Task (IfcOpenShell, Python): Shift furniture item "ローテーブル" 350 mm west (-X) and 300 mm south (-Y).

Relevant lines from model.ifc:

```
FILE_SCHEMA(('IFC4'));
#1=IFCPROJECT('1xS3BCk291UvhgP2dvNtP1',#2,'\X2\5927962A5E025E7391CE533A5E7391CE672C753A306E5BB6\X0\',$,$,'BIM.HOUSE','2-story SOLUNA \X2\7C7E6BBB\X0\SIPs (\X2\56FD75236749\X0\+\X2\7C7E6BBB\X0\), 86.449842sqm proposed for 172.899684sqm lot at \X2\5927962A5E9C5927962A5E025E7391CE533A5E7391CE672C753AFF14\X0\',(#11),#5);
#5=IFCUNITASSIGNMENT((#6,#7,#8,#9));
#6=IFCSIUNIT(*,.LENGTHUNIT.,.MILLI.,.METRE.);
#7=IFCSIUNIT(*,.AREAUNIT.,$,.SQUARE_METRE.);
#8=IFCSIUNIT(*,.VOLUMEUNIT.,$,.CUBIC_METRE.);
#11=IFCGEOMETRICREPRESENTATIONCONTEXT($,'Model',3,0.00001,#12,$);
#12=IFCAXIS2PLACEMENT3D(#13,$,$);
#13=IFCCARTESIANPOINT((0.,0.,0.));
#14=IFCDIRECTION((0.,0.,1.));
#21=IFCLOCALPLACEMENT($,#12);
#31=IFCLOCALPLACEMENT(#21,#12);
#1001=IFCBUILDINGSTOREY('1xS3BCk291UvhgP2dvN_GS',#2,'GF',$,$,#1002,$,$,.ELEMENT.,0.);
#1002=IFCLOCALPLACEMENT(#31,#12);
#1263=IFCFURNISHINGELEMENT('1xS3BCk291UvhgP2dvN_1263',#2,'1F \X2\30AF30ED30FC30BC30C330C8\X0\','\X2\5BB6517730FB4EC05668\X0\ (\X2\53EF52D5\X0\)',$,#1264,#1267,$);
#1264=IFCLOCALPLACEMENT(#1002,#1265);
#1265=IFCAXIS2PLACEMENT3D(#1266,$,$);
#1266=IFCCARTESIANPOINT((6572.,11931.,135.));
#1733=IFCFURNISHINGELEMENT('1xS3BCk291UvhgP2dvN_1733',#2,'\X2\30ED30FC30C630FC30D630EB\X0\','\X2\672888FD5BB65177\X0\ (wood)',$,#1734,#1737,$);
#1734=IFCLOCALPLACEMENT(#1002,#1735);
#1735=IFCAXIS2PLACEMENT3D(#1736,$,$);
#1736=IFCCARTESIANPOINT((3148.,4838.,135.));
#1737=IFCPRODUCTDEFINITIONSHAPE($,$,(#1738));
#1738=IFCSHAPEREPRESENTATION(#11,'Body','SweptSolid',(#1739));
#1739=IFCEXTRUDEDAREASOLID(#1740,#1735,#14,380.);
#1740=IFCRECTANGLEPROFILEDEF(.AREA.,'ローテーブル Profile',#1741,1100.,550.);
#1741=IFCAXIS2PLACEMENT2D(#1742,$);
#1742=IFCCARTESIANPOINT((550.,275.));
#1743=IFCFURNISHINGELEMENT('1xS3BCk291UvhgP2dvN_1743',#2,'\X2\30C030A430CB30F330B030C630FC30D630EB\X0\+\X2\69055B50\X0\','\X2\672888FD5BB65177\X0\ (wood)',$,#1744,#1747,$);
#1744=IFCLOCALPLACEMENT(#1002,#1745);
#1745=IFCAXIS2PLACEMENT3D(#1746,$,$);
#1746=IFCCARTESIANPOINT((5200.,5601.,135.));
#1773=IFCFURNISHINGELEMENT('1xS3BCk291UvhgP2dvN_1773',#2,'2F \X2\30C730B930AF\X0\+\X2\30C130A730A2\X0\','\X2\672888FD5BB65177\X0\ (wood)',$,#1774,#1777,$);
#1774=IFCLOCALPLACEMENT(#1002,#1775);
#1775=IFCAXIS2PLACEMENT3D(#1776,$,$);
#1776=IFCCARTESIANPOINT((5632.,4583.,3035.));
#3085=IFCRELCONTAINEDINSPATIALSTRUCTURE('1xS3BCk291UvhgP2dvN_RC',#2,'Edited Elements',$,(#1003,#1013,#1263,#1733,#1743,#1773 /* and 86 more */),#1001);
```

```python
import ifcopenshell
import ifcopenshell.api.geometry
import ifcopenshell.util.placement

model = ifcopenshell.open("model.ifc")

item = model.by_guid("1xS3BCk291UvhgP2dvN_1733")
matrix = ifcopenshell.util.placement.get_local_placement(item.ObjectPlacement)
matrix[0, 3] -= 350.0
matrix[1, 3] -= 300.0
ifcopenshell.api.geometry.edit_object_placement(model, product=item, matrix=matrix, is_si=False)

print(ifcopenshell.util.placement.get_local_placement(item.ObjectPlacement).round(3) + 0.0)

model.write("model_rev.ifc")
```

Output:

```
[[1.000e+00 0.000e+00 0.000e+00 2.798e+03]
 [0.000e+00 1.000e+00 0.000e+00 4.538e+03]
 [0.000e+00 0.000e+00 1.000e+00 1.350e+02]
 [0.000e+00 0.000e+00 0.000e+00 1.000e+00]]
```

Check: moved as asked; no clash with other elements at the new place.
